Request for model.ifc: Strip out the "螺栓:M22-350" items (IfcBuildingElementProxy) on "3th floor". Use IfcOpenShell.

First a look at what the model holds.

```python
import ifcopenshell
import ifcopenshell.util.element

model = ifcopenshell.open("model.ifc")
print(model.schema)
storey = next(s for s in model.by_type("IfcBuildingStorey") if s.Name == "3th floor")
proxies = [e for e in ifcopenshell.util.element.get_decomposition(storey) if e.is_a("IfcBuildingElementProxy")]
seen = {}
for e in proxies:
    element_type = ifcopenshell.util.element.get_type(e)
    name = element_type.Name if element_type not in (None, e) else None
    seen[name] = seen.get(name, 0) + 1
for name, count in sorted(seen.items(), key=str):
    print(count, "x", name)
```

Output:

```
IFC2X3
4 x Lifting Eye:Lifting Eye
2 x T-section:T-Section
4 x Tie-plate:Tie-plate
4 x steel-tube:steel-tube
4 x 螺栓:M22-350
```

```python
import ifcopenshell
import ifcopenshell.api.root
import ifcopenshell.util.element

model = ifcopenshell.open("model.ifc")

storey = next(s for s in model.by_type("IfcBuildingStorey") if s.Name == "3th floor")
proxies = [e for e in ifcopenshell.util.element.get_decomposition(storey) if e.is_a("IfcBuildingElementProxy")]
targets = [e for e in proxies if (t := ifcopenshell.util.element.get_type(e)) not in (None, e) and t.Name == "螺栓:M22-350"]

for e in targets:
    ifcopenshell.api.root.remove_product(model, product=e)
print(len(targets), "removed")

model.write("model_rev.ifc")
```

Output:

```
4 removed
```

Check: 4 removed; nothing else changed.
